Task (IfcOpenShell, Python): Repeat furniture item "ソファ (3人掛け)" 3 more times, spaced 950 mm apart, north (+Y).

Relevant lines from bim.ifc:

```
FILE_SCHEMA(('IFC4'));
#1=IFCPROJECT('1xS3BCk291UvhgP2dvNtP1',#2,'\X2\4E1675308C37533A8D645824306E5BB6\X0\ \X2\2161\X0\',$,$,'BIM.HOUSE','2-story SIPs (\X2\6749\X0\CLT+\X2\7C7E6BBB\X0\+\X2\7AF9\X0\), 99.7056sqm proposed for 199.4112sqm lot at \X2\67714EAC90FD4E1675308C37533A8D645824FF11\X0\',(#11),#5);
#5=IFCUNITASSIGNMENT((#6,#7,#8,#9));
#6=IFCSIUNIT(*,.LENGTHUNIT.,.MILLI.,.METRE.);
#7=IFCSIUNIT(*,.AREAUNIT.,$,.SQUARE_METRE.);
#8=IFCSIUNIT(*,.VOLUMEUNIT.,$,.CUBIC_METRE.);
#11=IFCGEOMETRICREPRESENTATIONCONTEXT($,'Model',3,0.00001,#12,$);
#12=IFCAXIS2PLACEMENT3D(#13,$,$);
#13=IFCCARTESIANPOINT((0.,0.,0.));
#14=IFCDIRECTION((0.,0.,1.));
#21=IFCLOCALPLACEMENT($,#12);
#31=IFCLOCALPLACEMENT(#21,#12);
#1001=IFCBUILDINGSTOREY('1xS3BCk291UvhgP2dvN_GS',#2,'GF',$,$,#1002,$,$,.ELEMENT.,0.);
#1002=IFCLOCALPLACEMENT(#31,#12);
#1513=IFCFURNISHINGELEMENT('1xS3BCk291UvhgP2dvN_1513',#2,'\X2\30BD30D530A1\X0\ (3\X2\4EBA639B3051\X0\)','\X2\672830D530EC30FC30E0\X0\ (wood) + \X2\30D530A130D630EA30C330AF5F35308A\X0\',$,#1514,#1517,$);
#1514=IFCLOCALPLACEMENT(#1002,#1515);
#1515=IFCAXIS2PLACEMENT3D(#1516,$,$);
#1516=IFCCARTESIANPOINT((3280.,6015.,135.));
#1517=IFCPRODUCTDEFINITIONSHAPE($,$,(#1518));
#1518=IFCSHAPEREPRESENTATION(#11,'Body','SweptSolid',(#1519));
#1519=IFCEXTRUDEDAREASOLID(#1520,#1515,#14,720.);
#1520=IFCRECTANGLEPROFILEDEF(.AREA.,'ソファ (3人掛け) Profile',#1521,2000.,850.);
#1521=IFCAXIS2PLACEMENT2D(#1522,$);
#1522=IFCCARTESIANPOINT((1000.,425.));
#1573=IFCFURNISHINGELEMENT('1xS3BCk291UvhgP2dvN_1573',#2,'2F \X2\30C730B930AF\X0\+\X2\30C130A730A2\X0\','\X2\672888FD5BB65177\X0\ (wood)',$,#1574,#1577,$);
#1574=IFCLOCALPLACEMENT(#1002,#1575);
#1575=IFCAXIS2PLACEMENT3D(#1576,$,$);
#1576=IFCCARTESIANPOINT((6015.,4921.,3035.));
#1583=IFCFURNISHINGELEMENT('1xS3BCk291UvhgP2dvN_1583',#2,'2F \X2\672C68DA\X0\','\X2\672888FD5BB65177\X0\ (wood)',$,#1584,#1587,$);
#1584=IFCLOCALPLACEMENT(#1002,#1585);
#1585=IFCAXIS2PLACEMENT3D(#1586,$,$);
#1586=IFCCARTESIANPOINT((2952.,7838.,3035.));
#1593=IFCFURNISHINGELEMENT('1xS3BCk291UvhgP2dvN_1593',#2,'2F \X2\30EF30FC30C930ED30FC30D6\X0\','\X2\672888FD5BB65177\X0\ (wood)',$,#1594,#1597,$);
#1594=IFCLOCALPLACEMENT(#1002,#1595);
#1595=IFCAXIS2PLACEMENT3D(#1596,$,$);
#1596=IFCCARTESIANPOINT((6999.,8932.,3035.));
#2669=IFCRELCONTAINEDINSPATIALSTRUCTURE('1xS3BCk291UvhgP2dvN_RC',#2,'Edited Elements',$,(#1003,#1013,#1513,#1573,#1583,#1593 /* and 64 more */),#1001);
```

```python
import numpy as np
import ifcopenshell
import ifcopenshell.api.geometry
import ifcopenshell.api.root
import ifcopenshell.util.element
import ifcopenshell.util.placement
import ifcopenshell.util.unit

model = ifcopenshell.open("bim.ifc")
unit_scale = ifcopenshell.util.unit.calculate_unit_scale(model)


def reuse_history(source, copy):
    """copy_class also copies each property set's owner history, people and application; keep the originals."""
    for rel in copy.IsDefinedBy:
        if rel.is_a("IfcRelDefinesByProperties") and (history := rel.RelatingPropertyDefinition.OwnerHistory):
            rel.RelatingPropertyDefinition.OwnerHistory = source.OwnerHistory
            ifcopenshell.util.element.remove_deep2(model, history)


source = model.by_guid("1xS3BCk291UvhgP2dvN_1513")
base = ifcopenshell.util.placement.get_local_placement(source.ObjectPlacement)
step = np.array([0.0, 1.0, 0.0]) * 0.95 / unit_scale

for i in range(1, 4):
    copy = ifcopenshell.api.root.copy_class(model, product=source)
    copy.Representation = ifcopenshell.util.element.copy_deep(
        model, source.Representation, exclude=["IfcGeometricRepresentationContext", "IfcRepresentationMap"]
    )
    reuse_history(source, copy)
    matrix = base.copy()
    matrix[:3, 3] += i * step
    print("added at", matrix[:3, 3].round(3) + 0.0)
    ifcopenshell.api.geometry.edit_object_placement(model, product=copy, matrix=matrix, is_si=False)

model.write("bim-out.ifc")
```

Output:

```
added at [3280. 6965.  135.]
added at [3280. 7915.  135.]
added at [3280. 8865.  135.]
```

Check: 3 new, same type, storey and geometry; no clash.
